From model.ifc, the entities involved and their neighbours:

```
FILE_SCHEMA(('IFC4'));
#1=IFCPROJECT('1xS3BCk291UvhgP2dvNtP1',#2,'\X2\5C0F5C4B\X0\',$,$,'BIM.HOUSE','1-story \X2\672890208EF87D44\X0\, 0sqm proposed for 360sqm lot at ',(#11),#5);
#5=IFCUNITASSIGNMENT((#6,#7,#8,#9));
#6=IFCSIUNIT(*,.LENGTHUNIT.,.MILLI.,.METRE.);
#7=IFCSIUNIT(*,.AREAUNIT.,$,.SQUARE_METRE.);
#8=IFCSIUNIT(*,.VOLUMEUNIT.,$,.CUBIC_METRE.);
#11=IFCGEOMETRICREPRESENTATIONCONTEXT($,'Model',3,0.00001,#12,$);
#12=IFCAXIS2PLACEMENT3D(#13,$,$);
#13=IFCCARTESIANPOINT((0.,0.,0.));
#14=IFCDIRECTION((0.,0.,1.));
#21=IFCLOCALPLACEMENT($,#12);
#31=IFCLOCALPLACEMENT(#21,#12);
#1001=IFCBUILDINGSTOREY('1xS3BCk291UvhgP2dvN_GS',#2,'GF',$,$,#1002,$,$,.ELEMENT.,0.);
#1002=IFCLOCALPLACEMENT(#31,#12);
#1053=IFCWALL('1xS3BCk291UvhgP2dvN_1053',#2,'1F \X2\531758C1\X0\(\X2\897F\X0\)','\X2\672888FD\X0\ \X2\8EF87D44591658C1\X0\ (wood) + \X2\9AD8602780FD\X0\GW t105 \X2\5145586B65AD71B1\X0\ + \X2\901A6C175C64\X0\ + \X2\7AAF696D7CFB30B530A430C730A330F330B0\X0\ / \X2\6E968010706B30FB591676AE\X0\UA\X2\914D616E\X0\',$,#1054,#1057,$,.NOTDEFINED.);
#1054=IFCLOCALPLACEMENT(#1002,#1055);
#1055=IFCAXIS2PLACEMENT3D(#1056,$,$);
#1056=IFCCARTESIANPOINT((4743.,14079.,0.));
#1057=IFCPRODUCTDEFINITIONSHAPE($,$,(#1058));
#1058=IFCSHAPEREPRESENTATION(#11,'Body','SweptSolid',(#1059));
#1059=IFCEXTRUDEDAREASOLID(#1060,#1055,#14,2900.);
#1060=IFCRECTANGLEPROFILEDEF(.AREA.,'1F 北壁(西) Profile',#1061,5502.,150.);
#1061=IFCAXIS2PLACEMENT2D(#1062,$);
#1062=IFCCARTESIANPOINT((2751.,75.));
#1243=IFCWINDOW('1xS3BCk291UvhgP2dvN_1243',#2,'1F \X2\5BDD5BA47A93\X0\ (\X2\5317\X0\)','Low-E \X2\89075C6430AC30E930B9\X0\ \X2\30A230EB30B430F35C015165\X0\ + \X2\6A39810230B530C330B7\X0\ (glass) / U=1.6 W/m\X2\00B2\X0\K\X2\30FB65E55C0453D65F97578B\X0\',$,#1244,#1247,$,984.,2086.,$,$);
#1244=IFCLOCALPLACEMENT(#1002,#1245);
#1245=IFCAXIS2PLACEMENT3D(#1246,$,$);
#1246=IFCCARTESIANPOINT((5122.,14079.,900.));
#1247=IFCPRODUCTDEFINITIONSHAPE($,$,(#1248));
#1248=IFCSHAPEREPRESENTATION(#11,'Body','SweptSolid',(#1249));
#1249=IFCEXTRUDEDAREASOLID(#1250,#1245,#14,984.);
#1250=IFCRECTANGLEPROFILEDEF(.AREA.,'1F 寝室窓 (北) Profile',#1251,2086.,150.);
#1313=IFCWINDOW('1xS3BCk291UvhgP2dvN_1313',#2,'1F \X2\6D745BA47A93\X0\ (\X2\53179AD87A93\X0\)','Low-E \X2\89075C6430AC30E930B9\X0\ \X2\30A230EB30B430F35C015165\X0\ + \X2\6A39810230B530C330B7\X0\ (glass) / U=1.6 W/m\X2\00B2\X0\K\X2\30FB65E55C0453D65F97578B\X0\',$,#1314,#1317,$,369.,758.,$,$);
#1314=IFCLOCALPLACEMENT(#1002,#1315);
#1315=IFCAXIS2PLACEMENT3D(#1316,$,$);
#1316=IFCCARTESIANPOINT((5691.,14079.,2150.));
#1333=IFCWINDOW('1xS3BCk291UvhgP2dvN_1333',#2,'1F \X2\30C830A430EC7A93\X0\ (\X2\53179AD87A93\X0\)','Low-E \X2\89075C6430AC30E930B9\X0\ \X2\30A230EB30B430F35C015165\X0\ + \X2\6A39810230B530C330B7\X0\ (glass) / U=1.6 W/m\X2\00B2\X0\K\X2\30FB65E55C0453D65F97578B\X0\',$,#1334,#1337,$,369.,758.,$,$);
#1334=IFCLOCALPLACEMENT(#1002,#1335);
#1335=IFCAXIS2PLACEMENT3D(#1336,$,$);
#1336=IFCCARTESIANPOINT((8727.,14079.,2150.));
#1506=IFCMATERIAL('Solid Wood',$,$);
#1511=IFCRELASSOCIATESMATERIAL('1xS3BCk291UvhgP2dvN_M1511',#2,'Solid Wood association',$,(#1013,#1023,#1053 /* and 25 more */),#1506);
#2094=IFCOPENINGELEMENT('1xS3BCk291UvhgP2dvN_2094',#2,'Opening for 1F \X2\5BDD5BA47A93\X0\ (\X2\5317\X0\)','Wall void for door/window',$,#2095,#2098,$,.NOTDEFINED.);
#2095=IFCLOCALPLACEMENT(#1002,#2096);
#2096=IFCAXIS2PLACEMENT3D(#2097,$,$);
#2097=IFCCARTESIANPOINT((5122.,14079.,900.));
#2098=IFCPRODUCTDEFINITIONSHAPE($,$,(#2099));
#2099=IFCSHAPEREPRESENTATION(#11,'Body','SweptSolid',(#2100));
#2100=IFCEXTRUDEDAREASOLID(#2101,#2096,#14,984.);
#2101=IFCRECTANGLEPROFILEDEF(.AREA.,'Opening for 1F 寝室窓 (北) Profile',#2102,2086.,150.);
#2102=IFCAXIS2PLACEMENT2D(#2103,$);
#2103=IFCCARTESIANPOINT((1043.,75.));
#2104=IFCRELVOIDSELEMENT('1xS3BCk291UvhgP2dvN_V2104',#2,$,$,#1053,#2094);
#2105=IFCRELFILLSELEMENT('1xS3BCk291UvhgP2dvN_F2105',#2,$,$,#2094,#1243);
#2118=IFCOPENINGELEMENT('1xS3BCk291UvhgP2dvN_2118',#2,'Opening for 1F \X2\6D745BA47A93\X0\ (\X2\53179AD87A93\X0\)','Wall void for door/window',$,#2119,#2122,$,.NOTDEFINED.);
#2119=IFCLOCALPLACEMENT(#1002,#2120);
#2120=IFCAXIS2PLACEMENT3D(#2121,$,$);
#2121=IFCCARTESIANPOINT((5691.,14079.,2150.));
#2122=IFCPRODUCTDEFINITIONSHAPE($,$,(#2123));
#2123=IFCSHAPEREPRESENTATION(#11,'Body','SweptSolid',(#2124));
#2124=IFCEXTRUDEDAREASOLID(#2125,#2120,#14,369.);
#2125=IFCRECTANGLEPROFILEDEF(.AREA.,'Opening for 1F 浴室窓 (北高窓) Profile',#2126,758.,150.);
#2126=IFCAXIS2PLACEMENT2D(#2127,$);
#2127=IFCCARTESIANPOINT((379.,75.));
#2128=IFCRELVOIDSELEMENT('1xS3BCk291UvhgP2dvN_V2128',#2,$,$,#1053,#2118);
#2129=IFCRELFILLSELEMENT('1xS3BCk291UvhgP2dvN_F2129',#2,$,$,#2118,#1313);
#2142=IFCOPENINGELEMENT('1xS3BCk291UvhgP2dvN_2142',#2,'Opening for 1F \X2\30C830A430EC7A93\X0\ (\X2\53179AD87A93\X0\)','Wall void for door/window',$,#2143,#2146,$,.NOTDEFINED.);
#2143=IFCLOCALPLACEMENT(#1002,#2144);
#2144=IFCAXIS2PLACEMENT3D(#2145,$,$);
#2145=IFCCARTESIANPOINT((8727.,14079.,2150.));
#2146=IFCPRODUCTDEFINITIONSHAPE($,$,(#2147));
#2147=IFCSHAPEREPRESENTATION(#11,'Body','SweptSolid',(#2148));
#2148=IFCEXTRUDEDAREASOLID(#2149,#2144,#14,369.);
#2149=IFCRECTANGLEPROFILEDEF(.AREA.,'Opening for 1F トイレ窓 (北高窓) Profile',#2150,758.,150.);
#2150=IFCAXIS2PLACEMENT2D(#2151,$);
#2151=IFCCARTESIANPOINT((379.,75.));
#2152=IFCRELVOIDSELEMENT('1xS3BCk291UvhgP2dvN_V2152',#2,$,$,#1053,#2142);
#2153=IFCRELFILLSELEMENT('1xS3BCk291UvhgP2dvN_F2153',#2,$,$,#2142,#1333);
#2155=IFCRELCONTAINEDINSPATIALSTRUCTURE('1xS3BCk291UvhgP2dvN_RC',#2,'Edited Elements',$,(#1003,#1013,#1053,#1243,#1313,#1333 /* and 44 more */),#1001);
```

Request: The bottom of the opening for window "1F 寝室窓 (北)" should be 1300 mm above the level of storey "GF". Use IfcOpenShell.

```python
import numpy as np
import ifcopenshell
import ifcopenshell.api.geometry
import ifcopenshell.geom
import ifcopenshell.util.element
import ifcopenshell.util.placement
import ifcopenshell.util.shape
import ifcopenshell.util.unit

model = ifcopenshell.open("model.ifc")
unit_scale = ifcopenshell.util.unit.calculate_unit_scale(model)

window = model.by_guid("1xS3BCk291UvhgP2dvN_1243")
opening = window.FillsVoids[0].RelatingOpeningElement
storey = ifcopenshell.util.element.get_container(window, ifc_class="IfcBuildingStorey")
level = ifcopenshell.util.placement.get_local_placement(storey.ObjectPlacement)[2, 3]

# The opening's origin need not be at the sill, so measure its lowest point.
shape = ifcopenshell.geom.create_shape(ifcopenshell.geom.settings(), opening)
bottom = ifcopenshell.util.shape.get_shape_bottom_elevation(shape, shape.geometry) / unit_scale
dz = level + 1.3 / unit_scale - bottom

shift = np.array([0.0, 0.0, dz])
# The window is not placed relative to its opening, so move both.
for product in (opening, window):
    matrix = ifcopenshell.util.placement.get_local_placement(product.ObjectPlacement)
    matrix[:3, 3] += shift
    ifcopenshell.api.geometry.edit_object_placement(model, product=product, matrix=matrix, is_si=False)

print(f"moved by {dz * unit_scale:+.3f} m")

model.write("model_edited.ifc")
```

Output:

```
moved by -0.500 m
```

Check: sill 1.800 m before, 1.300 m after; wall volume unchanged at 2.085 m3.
